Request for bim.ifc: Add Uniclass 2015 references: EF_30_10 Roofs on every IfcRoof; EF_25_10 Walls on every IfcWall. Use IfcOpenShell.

First a look at what the model holds.

```python
import ifcopenshell

model = ifcopenshell.open("bim.ifc")
print(model.schema)
print("classifications:", [c.Name for c in model.by_type("IfcClassification")])
for ifc_class in ("IfcDoor", "IfcRoof", "IfcStair", "IfcWall", "IfcWindow"):
    print(ifc_class, len(model.by_type(ifc_class)))
```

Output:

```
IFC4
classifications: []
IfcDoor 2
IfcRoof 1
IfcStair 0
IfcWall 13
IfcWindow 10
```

```python
import ifcopenshell
import ifcopenshell.api.classification

model = ifcopenshell.open("bim.ifc")

system = ifcopenshell.api.classification.add_classification(model, classification="Uniclass 2015")

codes = {
    "IfcRoof": ("EF_30_10", "Roofs"),
    "IfcWall": ("EF_25_10", "Walls"),
}
for ifc_class, (code, name) in codes.items():
    products = model.by_type(ifc_class)
    ifcopenshell.api.classification.add_reference(
        model, products=products, classification=system, identification=code, name=name
    )
    print(code, len(products))

model.write("bim_rev.ifc")
```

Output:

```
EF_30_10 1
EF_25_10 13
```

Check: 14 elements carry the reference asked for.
